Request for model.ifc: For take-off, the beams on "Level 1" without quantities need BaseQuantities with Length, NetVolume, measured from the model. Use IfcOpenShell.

First a look at what the model holds.

```python
import ifcopenshell
import ifcopenshell.util.element
import ifcopenshell.util.unit

model = ifcopenshell.open("model.ifc")
print(model.schema)
for unit_type in ("LENGTHUNIT", "AREAUNIT", "VOLUMEUNIT"):
    print(unit_type, ifcopenshell.util.unit.calculate_unit_scale(model, unit_type))
storey = next(s for s in model.by_type("IfcBuildingStorey") if s.Name == "Level 1")
beams = [e for e in ifcopenshell.util.element.get_decomposition(storey) if e.is_a("IfcBeam")]
for e in sorted(beams, key=lambda e: e.id()):
    print(e.id(), e.is_a(), e.Name, list(ifcopenshell.util.element.get_psets(e, qtos_only=True)), sep=" | ")
```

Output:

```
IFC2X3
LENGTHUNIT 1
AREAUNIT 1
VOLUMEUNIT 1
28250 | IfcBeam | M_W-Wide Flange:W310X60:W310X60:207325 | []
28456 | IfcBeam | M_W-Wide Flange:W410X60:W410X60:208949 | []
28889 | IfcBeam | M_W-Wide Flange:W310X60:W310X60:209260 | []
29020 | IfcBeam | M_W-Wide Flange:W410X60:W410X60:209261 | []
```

```python
import ifcopenshell
import ifcopenshell.api.pset
import ifcopenshell.geom
import ifcopenshell.util.element
import ifcopenshell.util.shape
import ifcopenshell.util.unit

model = ifcopenshell.open("model.ifc")
unit_scale = ifcopenshell.util.unit.calculate_unit_scale(model)
volume_scale = ifcopenshell.util.unit.calculate_unit_scale(model, "VOLUMEUNIT")
settings = ifcopenshell.geom.settings()

storey = next(s for s in model.by_type("IfcBuildingStorey") if s.Name == "Level 1")
beams = [e for e in ifcopenshell.util.element.get_decomposition(storey) if e.is_a("IfcBeam")]

for e in sorted(beams, key=lambda e: e.id()):
    if ifcopenshell.util.element.get_psets(e, qtos_only=True, should_inherit=False):
        continue
    # Geometry comes back in metres, in the element's own axes.
    shape = ifcopenshell.geom.create_shape(settings, e)
    values = {
        "Length": ifcopenshell.util.shape.get_max_xyz(shape.geometry) / unit_scale,
        "NetVolume": ifcopenshell.util.shape.get_volume(shape.geometry) / volume_scale,
    }
    qto = ifcopenshell.api.pset.add_qto(model, product=e, name="BaseQuantities")
    ifcopenshell.api.pset.edit_qto(model, qto=qto, properties=values)
    print(e.id(), {k: round(v, 3) for k, v in values.items()})

model.write("model_edited.ifc")
```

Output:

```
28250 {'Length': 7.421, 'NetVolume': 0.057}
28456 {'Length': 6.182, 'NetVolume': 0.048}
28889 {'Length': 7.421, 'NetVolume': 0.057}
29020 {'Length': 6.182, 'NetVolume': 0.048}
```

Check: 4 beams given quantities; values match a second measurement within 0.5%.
